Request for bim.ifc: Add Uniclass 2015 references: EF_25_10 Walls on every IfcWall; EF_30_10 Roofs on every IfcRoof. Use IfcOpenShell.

First a look at what the model holds.

```python
import ifcopenshell

model = ifcopenshell.open("bim.ifc")
print(model.schema)
print("classifications:", [c.Name for c in model.by_type("IfcClassification")])
for ifc_class in ("IfcDoor", "IfcRoof", "IfcStair", "IfcWall", "IfcWindow"):
    print(ifc_class, len(model.by_type(ifc_class)))
```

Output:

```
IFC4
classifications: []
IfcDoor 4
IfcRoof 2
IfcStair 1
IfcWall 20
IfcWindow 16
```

```python
import ifcopenshell
import ifcopenshell.api.classification

model = ifcopenshell.open("bim.ifc")

system = ifcopenshell.api.classification.add_classification(model, classification="Uniclass 2015")

codes = {
    "IfcWall": ("EF_25_10", "Walls"),
    "IfcRoof": ("EF_30_10", "Roofs"),
}
for ifc_class, (code, name) in codes.items():
    products = model.by_type(ifc_class)
    ifcopenshell.api.classification.add_reference(
        model, products=products, classification=system, identification=code, name=name
    )
    print(code, len(products))

model.write("bim-out.ifc")
```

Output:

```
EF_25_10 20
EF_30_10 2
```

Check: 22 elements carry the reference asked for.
